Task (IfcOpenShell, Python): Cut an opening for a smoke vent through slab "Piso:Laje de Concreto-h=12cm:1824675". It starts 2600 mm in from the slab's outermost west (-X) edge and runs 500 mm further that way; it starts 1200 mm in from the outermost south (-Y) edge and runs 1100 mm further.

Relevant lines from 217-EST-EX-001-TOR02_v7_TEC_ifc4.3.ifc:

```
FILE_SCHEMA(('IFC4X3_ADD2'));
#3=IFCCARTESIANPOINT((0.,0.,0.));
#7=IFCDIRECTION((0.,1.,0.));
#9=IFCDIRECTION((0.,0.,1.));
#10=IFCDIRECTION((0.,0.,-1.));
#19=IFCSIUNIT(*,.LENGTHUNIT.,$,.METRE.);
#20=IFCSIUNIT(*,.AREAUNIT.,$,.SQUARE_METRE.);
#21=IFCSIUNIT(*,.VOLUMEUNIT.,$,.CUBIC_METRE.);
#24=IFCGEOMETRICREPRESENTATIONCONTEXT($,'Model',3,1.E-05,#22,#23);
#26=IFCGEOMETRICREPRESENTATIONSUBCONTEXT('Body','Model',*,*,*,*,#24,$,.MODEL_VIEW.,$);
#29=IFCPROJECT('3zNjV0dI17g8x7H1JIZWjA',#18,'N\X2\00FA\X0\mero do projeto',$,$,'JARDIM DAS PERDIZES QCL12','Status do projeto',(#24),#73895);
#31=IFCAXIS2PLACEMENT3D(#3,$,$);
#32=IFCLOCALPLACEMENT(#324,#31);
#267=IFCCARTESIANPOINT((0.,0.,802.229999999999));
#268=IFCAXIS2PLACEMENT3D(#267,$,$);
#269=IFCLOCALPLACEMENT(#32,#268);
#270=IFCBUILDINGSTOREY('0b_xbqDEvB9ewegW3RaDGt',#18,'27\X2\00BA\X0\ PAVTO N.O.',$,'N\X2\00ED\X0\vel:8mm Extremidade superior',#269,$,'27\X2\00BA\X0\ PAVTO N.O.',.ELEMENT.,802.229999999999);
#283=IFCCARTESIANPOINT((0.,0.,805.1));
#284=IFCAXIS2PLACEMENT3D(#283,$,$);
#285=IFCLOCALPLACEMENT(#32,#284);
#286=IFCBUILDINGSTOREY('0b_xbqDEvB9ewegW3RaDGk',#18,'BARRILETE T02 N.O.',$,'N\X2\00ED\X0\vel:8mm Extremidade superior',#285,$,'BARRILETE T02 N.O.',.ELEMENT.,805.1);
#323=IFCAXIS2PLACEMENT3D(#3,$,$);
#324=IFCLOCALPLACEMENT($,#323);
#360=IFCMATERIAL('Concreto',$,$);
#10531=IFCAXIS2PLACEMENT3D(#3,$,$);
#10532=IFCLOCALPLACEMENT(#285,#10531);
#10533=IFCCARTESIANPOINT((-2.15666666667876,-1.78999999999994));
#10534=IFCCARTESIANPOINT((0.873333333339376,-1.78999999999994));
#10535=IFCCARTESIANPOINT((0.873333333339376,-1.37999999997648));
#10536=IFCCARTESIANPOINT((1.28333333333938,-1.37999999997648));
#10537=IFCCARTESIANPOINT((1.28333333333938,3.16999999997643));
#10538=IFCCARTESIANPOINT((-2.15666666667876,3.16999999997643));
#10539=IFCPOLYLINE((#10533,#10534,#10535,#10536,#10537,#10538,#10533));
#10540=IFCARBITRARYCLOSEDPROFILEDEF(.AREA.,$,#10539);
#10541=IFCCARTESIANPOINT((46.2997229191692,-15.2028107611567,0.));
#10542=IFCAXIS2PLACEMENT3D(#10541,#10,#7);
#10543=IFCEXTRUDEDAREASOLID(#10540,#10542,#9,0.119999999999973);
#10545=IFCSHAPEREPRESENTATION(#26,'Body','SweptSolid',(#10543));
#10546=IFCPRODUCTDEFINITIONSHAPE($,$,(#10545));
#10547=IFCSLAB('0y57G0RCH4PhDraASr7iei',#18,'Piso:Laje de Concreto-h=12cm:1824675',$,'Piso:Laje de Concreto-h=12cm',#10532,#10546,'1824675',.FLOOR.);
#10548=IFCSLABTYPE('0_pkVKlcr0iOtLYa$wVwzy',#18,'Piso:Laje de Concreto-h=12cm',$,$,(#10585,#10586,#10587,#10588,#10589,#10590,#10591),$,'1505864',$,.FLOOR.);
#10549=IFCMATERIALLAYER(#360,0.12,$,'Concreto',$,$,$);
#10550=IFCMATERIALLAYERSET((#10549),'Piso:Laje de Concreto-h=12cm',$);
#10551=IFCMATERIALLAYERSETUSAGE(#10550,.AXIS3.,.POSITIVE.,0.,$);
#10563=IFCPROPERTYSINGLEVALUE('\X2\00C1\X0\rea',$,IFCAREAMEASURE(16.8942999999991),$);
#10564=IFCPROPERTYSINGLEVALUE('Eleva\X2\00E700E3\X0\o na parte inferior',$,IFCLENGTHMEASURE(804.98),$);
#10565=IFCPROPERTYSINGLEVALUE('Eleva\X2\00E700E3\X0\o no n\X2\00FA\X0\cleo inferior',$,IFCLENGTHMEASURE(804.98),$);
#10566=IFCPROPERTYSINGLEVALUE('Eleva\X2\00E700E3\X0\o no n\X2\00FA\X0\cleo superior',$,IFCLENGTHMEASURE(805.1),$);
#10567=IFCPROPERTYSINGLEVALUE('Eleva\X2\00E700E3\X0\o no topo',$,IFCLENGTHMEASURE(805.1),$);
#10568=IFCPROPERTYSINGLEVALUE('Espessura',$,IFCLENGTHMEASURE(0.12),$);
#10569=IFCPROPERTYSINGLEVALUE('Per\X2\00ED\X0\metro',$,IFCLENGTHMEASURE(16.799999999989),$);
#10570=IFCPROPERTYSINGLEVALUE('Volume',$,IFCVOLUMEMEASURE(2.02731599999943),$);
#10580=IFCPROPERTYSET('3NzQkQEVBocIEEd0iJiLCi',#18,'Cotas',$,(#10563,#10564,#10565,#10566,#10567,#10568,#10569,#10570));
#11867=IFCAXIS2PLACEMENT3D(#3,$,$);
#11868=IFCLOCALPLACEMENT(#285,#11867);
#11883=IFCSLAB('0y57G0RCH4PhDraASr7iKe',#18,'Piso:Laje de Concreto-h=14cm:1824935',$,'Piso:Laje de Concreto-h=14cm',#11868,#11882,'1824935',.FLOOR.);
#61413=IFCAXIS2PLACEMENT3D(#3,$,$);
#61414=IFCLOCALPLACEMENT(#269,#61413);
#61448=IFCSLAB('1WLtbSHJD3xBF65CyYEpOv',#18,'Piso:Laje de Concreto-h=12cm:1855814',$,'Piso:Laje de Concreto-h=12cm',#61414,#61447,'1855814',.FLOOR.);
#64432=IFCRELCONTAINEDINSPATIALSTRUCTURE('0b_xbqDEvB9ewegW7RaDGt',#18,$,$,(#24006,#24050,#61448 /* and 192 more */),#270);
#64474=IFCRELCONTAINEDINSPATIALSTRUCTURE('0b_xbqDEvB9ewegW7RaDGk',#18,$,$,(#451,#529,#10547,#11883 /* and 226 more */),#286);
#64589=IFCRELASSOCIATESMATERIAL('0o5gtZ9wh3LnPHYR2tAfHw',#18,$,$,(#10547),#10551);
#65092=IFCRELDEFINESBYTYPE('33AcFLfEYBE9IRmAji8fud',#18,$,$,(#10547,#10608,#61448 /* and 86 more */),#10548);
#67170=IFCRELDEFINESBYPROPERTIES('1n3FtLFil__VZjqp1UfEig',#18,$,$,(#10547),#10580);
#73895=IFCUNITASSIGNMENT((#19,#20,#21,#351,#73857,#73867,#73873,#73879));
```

```python
import numpy as np
import ifcopenshell
import ifcopenshell.api.feature
import ifcopenshell.api.geometry
import ifcopenshell.api.pset
import ifcopenshell.api.root
import ifcopenshell.geom
import ifcopenshell.util.element
import ifcopenshell.util.placement
import ifcopenshell.util.representation
import ifcopenshell.util.shape
import ifcopenshell.util.unit

model = ifcopenshell.open("217-EST-EX-001-TOR02_v7_TEC_ifc4.3.ifc")
unit_scale = ifcopenshell.util.unit.calculate_unit_scale(model)
area_scale = ifcopenshell.util.unit.calculate_unit_scale(model, "AREAUNIT")
volume_scale = ifcopenshell.util.unit.calculate_unit_scale(model, "VOLUMEUNIT")
settings = ifcopenshell.geom.settings()


def volume(element):
    """Net volume in cubic metres, openings subtracted."""
    shape = ifcopenshell.geom.create_shape(settings, element)
    return ifcopenshell.util.shape.get_volume(shape.geometry)


slab = model.by_guid("0y57G0RCH4PhDraASr7iei")
before = volume(slab)

# Extent in the slab's own axes, in metres. The edges named are its -X and -Y sides.
slab_shape = ifcopenshell.geom.create_shape(settings, slab)
vertices = ifcopenshell.util.shape.get_vertices(slab_shape.geometry)
x_min, y_min, bottom = vertices.min(axis=0)
top = vertices[:, 2].max()

opening = ifcopenshell.api.root.create_entity(model, ifc_class="IfcOpeningElement", name="Smoke vent opening", predefined_type="OPENING")
context = ifcopenshell.util.representation.get_context(model, "Model", "Body", "MODEL_VIEW")
width, depth = 0.5, 1.1
outline = [(0.0, 0.0), (width, 0.0), (width, depth), (0.0, depth), (0.0, 0.0)]
# Overshoot both faces by 50 mm so the cut is clean.
shape = ifcopenshell.api.geometry.add_slab_representation(
    model, context=context, depth=top - bottom + 0.1, polyline=outline
)
ifcopenshell.api.geometry.assign_representation(model, product=opening, representation=shape)

matrix = ifcopenshell.util.placement.get_local_placement(slab.ObjectPlacement)
matrix[:, 3] = matrix @ np.append(np.array([x_min + 2.6, y_min + 1.2, bottom - 0.05]) / unit_scale, 1.0)
ifcopenshell.api.geometry.edit_object_placement(model, product=opening, matrix=matrix, is_si=False)
ifcopenshell.api.feature.add_feature(model, feature=opening, element=slab)

after = volume(slab)

# Update the slab's stored quantities.
pset = model.by_id(ifcopenshell.util.element.get_pset(slab, "Cotas", should_inherit=False)["id"])
ifcopenshell.api.pset.edit_pset(model, pset=pset, properties={
    "Área": model.create_entity("IfcAreaMeasure", after / (top - bottom) / area_scale),
    "Volume": model.create_entity("IfcVolumeMeasure", after / volume_scale),
})

print(f"slab volume {before:.3f} -> {after:.3f} m3")

model.write("217-EST-EX-001-TOR02_v7_TEC_ifc4.3_edited.ifc")
```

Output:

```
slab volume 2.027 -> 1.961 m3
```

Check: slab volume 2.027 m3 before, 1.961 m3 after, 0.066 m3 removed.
